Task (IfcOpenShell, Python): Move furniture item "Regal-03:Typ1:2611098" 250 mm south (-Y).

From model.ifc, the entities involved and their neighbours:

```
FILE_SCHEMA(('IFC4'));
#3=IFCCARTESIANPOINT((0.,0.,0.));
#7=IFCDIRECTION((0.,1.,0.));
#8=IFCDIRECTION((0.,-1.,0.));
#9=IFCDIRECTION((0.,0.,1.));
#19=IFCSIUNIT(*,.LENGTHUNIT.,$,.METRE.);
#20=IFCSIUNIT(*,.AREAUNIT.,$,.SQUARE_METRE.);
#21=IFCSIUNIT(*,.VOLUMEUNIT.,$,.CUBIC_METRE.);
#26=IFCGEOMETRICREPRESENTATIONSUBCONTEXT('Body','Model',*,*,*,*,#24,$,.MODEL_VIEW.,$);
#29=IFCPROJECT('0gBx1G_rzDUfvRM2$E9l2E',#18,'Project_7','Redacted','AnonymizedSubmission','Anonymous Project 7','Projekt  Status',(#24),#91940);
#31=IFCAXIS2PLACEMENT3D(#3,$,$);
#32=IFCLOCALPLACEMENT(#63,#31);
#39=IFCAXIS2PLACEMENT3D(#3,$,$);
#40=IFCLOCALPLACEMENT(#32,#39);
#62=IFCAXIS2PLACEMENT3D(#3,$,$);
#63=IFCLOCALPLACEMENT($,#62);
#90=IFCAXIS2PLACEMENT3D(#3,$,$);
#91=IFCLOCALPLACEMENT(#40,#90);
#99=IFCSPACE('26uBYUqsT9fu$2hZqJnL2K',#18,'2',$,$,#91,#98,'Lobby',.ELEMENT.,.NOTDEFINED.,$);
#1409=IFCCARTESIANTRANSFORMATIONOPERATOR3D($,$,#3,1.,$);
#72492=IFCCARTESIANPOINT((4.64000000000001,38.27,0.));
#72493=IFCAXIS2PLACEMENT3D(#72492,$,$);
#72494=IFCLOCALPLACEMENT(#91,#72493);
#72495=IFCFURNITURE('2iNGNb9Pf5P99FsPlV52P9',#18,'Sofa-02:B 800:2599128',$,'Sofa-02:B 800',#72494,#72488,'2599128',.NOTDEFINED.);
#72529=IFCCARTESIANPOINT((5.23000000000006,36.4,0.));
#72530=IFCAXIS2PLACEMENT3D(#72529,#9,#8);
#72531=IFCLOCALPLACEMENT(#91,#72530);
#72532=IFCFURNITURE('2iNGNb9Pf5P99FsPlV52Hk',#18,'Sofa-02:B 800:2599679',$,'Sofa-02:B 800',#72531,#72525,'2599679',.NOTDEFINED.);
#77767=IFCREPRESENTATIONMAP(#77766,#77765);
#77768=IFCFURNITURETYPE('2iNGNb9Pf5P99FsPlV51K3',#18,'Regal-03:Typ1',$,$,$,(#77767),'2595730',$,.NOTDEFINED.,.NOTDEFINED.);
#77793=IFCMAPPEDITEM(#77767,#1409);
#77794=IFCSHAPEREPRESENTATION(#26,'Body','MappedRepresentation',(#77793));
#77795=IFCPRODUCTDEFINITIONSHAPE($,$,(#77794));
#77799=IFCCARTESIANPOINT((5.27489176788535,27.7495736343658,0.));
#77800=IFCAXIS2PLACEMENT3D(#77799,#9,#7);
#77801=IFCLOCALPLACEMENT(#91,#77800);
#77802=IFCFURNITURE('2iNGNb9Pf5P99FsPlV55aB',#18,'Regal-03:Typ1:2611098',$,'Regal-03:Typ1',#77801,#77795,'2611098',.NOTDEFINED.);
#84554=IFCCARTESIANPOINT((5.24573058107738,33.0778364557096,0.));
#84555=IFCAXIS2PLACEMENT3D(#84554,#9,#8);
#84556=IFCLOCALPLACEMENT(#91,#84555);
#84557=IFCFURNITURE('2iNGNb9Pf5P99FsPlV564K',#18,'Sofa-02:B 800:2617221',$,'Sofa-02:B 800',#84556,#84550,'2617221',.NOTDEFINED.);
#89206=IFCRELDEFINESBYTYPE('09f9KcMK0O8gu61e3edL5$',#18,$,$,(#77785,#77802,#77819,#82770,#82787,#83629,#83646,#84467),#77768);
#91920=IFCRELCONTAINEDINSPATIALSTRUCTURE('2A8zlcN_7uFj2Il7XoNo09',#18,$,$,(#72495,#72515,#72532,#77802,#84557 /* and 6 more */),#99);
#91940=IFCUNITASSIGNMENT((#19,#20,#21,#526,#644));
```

```python
import ifcopenshell
import ifcopenshell.api.geometry
import ifcopenshell.util.placement
import ifcopenshell.util.unit

model = ifcopenshell.open("model.ifc")
unit_scale = ifcopenshell.util.unit.calculate_unit_scale(model)

item = model.by_guid("2iNGNb9Pf5P99FsPlV55aB")
matrix = ifcopenshell.util.placement.get_local_placement(item.ObjectPlacement)
matrix[1, 3] -= 0.25 / unit_scale
ifcopenshell.api.geometry.edit_object_placement(model, product=item, matrix=matrix, is_si=False)

print(ifcopenshell.util.placement.get_local_placement(item.ObjectPlacement).round(3) + 0.0)

model.write("model_updated.ifc")
```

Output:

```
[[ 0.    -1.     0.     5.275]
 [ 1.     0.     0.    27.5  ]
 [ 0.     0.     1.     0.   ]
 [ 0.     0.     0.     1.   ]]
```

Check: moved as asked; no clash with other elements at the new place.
